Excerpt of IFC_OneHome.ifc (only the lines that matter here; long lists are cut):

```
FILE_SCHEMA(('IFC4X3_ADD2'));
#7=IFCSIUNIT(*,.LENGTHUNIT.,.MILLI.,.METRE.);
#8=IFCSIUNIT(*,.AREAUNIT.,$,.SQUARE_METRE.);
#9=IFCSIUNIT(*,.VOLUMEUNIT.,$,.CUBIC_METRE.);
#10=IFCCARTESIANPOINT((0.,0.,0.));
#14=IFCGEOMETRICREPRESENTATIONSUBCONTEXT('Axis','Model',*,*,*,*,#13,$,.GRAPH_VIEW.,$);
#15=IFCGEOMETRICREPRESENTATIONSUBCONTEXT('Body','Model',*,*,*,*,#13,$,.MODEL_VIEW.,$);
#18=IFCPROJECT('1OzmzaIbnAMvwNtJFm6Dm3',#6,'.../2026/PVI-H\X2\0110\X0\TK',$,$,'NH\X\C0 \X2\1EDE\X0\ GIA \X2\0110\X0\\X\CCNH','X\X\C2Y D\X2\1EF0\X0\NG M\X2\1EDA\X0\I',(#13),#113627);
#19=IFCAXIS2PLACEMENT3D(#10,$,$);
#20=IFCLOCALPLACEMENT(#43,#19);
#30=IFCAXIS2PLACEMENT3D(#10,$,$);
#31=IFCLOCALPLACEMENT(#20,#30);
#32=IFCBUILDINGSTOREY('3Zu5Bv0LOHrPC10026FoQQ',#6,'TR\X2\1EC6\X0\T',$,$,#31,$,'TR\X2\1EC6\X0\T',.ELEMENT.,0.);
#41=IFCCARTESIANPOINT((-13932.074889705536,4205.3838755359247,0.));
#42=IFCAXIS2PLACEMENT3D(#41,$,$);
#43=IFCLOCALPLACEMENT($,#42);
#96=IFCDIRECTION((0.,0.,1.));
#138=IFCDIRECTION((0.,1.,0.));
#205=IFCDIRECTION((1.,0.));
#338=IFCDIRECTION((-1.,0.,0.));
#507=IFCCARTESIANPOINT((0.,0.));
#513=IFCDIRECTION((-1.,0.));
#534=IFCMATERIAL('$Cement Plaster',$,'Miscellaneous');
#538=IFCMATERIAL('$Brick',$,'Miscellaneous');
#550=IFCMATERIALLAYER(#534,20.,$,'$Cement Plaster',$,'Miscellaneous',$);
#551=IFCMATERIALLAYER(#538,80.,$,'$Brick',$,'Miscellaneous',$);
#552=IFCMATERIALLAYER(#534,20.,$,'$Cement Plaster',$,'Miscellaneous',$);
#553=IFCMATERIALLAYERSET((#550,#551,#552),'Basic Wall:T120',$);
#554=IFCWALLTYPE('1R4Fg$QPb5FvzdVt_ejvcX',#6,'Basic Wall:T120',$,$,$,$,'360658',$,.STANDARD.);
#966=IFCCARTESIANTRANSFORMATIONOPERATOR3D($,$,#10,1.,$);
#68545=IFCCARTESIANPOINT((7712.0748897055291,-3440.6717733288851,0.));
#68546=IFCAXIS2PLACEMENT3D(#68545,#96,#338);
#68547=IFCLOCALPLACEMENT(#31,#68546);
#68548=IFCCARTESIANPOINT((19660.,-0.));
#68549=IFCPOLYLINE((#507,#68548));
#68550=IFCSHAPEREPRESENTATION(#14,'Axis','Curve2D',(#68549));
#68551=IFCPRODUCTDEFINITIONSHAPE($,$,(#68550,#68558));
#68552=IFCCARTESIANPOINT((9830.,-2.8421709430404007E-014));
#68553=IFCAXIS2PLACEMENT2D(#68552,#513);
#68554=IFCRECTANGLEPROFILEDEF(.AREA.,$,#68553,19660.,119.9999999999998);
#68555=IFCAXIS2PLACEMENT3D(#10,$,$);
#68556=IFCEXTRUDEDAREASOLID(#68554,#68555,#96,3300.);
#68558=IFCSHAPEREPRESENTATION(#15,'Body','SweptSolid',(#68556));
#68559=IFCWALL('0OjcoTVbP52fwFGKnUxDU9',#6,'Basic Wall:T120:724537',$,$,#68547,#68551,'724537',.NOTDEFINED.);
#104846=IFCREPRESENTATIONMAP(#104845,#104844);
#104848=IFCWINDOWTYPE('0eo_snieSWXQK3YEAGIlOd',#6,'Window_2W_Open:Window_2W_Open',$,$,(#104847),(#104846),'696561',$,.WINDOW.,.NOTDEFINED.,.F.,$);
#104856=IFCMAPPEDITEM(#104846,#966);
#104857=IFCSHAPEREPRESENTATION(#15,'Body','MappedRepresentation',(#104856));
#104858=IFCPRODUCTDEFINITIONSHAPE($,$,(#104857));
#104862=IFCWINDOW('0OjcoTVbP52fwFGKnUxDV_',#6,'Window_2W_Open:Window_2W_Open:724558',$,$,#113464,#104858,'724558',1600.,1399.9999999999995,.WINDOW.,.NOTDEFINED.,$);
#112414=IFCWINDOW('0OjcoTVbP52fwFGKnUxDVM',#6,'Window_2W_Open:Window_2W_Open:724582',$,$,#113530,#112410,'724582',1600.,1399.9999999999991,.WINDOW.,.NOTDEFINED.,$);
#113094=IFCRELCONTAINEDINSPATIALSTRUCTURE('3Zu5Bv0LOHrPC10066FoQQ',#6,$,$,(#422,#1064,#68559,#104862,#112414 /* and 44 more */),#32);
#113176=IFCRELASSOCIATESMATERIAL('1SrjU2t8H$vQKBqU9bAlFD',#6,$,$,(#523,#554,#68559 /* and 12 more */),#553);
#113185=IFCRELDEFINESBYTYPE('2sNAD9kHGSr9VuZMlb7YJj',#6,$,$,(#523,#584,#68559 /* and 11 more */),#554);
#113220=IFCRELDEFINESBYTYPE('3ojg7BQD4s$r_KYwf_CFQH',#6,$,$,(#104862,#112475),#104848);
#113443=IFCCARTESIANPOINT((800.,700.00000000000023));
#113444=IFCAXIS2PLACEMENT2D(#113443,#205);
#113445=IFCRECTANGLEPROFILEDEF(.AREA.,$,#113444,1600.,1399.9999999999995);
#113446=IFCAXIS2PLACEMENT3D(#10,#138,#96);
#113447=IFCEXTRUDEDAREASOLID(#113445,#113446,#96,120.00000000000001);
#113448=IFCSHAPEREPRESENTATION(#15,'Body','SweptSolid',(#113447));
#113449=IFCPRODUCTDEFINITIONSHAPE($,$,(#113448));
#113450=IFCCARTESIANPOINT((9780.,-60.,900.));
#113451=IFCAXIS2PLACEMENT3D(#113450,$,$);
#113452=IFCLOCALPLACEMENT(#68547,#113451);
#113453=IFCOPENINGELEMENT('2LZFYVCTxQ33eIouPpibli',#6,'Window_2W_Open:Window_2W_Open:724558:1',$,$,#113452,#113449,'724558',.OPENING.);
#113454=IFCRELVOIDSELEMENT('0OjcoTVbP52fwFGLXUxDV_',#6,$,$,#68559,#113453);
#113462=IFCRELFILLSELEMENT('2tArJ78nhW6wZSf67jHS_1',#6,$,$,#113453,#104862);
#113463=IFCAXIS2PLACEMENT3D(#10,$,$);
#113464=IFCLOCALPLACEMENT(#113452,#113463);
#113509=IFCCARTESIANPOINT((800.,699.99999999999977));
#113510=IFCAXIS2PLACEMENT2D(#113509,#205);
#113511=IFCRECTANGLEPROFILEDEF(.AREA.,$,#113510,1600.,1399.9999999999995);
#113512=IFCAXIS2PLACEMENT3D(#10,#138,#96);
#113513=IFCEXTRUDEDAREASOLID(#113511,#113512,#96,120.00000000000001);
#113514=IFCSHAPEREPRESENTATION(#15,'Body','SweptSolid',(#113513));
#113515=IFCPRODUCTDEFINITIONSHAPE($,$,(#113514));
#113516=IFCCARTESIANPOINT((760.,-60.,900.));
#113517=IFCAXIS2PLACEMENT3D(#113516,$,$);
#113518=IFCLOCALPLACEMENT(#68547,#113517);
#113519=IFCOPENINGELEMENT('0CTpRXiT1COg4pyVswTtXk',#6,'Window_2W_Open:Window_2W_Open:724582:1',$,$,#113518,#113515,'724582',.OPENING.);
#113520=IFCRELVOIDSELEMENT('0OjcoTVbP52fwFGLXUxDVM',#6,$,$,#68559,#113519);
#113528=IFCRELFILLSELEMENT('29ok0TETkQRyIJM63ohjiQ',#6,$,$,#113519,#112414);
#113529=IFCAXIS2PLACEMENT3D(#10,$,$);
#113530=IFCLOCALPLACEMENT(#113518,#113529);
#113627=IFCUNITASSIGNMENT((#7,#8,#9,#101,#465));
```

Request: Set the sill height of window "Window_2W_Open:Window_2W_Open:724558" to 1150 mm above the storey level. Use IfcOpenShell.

```python
import numpy as np
import ifcopenshell
import ifcopenshell.api.geometry
import ifcopenshell.geom
import ifcopenshell.util.element
import ifcopenshell.util.placement
import ifcopenshell.util.shape
import ifcopenshell.util.unit

model = ifcopenshell.open("IFC_OneHome.ifc")
unit_scale = ifcopenshell.util.unit.calculate_unit_scale(model)

window = model.by_id(104862)
opening = window.FillsVoids[0].RelatingOpeningElement
storey = ifcopenshell.util.element.get_container(window, ifc_class="IfcBuildingStorey")
level = ifcopenshell.util.placement.get_local_placement(storey.ObjectPlacement)[2, 3]

# The opening's origin need not be at the sill, so measure its lowest point.
shape = ifcopenshell.geom.create_shape(ifcopenshell.geom.settings(), opening)
bottom = ifcopenshell.util.shape.get_shape_bottom_elevation(shape, shape.geometry) / unit_scale
dz = level + 1.15 / unit_scale - bottom

shift = np.array([0.0, 0.0, dz])
# The window is placed relative to its opening, so it follows when the opening moves.
matrix = ifcopenshell.util.placement.get_local_placement(opening.ObjectPlacement)
matrix[:3, 3] += shift
ifcopenshell.api.geometry.edit_object_placement(
    model, product=opening, matrix=matrix, is_si=False, should_transform_children=True
)

print(f"moved by {dz * unit_scale:+.3f} m")

model.write("IFC_OneHome_v2.ifc")
```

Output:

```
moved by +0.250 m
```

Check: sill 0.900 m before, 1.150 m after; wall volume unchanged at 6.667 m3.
